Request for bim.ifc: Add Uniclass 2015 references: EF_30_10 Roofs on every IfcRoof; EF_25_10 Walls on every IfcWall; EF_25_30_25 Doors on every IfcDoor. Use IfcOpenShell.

First a look at what the model holds.

```python
import ifcopenshell

model = ifcopenshell.open("bim.ifc")
print(model.schema)
print("classifications:", [c.Name for c in model.by_type("IfcClassification")])
for ifc_class in ("IfcDoor", "IfcRoof", "IfcStair", "IfcWall", "IfcWindow"):
    print(ifc_class, len(model.by_type(ifc_class)))
```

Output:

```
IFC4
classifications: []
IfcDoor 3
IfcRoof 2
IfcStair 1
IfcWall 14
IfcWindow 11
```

```python
import ifcopenshell
import ifcopenshell.api.classification

model = ifcopenshell.open("bim.ifc")

system = ifcopenshell.api.classification.add_classification(model, classification="Uniclass 2015")

codes = {
    "IfcRoof": ("EF_30_10", "Roofs"),
    "IfcWall": ("EF_25_10", "Walls"),
    "IfcDoor": ("EF_25_30_25", "Doors"),
}
for ifc_class, (code, name) in codes.items():
    products = model.by_type(ifc_class)
    ifcopenshell.api.classification.add_reference(
        model, products=products, classification=system, identification=code, name=name
    )
    print(code, len(products))

model.write("bim_rev.ifc")
```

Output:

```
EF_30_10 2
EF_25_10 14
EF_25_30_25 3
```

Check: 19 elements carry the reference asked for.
